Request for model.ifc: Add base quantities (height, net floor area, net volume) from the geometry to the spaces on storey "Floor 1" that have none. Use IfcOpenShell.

First a look at what the model holds.

```python
import ifcopenshell
import ifcopenshell.util.element
import ifcopenshell.util.unit

model = ifcopenshell.open("model.ifc")
print(model.schema)
for unit_type in ("LENGTHUNIT", "AREAUNIT", "VOLUMEUNIT"):
    print(unit_type, ifcopenshell.util.unit.calculate_unit_scale(model, unit_type))
storey = next(s for s in model.by_type("IfcBuildingStorey") if s.Name == "Floor 1")
spaces = [e for e in ifcopenshell.util.element.get_decomposition(storey) if e.is_a("IfcSpace")]
for e in sorted(spaces, key=lambda e: e.id()):
    print(e.id(), e.is_a(), e.Name, list(ifcopenshell.util.element.get_psets(e, qtos_only=True)), sep=" | ")
```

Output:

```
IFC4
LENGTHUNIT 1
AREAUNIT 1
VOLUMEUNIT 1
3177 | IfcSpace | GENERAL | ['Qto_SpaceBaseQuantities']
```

```python
import ifcopenshell
import ifcopenshell.api.pset
import ifcopenshell.geom
import ifcopenshell.util.element
import ifcopenshell.util.shape
import ifcopenshell.util.unit

model = ifcopenshell.open("model.ifc")
unit_scale = ifcopenshell.util.unit.calculate_unit_scale(model)
area_scale = ifcopenshell.util.unit.calculate_unit_scale(model, "AREAUNIT")
volume_scale = ifcopenshell.util.unit.calculate_unit_scale(model, "VOLUMEUNIT")
settings = ifcopenshell.geom.settings()

storey = next(s for s in model.by_type("IfcBuildingStorey") if s.Name == "Floor 1")
spaces = [e for e in ifcopenshell.util.element.get_decomposition(storey) if e.is_a("IfcSpace")]

for e in sorted(spaces, key=lambda e: e.id()):
    if ifcopenshell.util.element.get_psets(e, qtos_only=True, should_inherit=False):
        continue
    # Geometry comes back in metres, in the element's own axes.
    shape = ifcopenshell.geom.create_shape(settings, e)
    values = {
        "Height": ifcopenshell.util.shape.get_z(shape.geometry) / unit_scale,
        "NetFloorArea": ifcopenshell.util.shape.get_footprint_area(shape.geometry) / area_scale,
        "NetVolume": ifcopenshell.util.shape.get_volume(shape.geometry) / volume_scale,
    }
    qto = ifcopenshell.api.pset.add_qto(model, product=e, name="Qto_SpaceBaseQuantities")
    ifcopenshell.api.pset.edit_qto(model, qto=qto, properties=values)
    print(e.id(), {k: round(v, 3) for k, v in values.items()})

model.write("model_updated.ifc")
```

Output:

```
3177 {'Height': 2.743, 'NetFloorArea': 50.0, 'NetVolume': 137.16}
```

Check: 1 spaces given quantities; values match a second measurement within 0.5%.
